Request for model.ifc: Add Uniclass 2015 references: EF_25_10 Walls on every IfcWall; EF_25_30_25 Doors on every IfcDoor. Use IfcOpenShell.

First a look at what the model holds.

```python
import ifcopenshell

model = ifcopenshell.open("model.ifc")
print(model.schema)
print("classifications:", [c.Name for c in model.by_type("IfcClassification")])
for ifc_class in ("IfcDoor", "IfcRoof", "IfcStair", "IfcWall", "IfcWindow"):
    print(ifc_class, len(model.by_type(ifc_class)))
```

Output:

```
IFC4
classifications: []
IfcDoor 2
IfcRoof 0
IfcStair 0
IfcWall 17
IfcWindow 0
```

```python
import ifcopenshell
import ifcopenshell.api.classification

model = ifcopenshell.open("model.ifc")

system = ifcopenshell.api.classification.add_classification(model, classification="Uniclass 2015")

codes = {
    "IfcWall": ("EF_25_10", "Walls"),
    "IfcDoor": ("EF_25_30_25", "Doors"),
}
for ifc_class, (code, name) in codes.items():
    products = model.by_type(ifc_class)
    ifcopenshell.api.classification.add_reference(
        model, products=products, classification=system, identification=code, name=name
    )
    print(code, len(products))

model.write("model_rev.ifc")
```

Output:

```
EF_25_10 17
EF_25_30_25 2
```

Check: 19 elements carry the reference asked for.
